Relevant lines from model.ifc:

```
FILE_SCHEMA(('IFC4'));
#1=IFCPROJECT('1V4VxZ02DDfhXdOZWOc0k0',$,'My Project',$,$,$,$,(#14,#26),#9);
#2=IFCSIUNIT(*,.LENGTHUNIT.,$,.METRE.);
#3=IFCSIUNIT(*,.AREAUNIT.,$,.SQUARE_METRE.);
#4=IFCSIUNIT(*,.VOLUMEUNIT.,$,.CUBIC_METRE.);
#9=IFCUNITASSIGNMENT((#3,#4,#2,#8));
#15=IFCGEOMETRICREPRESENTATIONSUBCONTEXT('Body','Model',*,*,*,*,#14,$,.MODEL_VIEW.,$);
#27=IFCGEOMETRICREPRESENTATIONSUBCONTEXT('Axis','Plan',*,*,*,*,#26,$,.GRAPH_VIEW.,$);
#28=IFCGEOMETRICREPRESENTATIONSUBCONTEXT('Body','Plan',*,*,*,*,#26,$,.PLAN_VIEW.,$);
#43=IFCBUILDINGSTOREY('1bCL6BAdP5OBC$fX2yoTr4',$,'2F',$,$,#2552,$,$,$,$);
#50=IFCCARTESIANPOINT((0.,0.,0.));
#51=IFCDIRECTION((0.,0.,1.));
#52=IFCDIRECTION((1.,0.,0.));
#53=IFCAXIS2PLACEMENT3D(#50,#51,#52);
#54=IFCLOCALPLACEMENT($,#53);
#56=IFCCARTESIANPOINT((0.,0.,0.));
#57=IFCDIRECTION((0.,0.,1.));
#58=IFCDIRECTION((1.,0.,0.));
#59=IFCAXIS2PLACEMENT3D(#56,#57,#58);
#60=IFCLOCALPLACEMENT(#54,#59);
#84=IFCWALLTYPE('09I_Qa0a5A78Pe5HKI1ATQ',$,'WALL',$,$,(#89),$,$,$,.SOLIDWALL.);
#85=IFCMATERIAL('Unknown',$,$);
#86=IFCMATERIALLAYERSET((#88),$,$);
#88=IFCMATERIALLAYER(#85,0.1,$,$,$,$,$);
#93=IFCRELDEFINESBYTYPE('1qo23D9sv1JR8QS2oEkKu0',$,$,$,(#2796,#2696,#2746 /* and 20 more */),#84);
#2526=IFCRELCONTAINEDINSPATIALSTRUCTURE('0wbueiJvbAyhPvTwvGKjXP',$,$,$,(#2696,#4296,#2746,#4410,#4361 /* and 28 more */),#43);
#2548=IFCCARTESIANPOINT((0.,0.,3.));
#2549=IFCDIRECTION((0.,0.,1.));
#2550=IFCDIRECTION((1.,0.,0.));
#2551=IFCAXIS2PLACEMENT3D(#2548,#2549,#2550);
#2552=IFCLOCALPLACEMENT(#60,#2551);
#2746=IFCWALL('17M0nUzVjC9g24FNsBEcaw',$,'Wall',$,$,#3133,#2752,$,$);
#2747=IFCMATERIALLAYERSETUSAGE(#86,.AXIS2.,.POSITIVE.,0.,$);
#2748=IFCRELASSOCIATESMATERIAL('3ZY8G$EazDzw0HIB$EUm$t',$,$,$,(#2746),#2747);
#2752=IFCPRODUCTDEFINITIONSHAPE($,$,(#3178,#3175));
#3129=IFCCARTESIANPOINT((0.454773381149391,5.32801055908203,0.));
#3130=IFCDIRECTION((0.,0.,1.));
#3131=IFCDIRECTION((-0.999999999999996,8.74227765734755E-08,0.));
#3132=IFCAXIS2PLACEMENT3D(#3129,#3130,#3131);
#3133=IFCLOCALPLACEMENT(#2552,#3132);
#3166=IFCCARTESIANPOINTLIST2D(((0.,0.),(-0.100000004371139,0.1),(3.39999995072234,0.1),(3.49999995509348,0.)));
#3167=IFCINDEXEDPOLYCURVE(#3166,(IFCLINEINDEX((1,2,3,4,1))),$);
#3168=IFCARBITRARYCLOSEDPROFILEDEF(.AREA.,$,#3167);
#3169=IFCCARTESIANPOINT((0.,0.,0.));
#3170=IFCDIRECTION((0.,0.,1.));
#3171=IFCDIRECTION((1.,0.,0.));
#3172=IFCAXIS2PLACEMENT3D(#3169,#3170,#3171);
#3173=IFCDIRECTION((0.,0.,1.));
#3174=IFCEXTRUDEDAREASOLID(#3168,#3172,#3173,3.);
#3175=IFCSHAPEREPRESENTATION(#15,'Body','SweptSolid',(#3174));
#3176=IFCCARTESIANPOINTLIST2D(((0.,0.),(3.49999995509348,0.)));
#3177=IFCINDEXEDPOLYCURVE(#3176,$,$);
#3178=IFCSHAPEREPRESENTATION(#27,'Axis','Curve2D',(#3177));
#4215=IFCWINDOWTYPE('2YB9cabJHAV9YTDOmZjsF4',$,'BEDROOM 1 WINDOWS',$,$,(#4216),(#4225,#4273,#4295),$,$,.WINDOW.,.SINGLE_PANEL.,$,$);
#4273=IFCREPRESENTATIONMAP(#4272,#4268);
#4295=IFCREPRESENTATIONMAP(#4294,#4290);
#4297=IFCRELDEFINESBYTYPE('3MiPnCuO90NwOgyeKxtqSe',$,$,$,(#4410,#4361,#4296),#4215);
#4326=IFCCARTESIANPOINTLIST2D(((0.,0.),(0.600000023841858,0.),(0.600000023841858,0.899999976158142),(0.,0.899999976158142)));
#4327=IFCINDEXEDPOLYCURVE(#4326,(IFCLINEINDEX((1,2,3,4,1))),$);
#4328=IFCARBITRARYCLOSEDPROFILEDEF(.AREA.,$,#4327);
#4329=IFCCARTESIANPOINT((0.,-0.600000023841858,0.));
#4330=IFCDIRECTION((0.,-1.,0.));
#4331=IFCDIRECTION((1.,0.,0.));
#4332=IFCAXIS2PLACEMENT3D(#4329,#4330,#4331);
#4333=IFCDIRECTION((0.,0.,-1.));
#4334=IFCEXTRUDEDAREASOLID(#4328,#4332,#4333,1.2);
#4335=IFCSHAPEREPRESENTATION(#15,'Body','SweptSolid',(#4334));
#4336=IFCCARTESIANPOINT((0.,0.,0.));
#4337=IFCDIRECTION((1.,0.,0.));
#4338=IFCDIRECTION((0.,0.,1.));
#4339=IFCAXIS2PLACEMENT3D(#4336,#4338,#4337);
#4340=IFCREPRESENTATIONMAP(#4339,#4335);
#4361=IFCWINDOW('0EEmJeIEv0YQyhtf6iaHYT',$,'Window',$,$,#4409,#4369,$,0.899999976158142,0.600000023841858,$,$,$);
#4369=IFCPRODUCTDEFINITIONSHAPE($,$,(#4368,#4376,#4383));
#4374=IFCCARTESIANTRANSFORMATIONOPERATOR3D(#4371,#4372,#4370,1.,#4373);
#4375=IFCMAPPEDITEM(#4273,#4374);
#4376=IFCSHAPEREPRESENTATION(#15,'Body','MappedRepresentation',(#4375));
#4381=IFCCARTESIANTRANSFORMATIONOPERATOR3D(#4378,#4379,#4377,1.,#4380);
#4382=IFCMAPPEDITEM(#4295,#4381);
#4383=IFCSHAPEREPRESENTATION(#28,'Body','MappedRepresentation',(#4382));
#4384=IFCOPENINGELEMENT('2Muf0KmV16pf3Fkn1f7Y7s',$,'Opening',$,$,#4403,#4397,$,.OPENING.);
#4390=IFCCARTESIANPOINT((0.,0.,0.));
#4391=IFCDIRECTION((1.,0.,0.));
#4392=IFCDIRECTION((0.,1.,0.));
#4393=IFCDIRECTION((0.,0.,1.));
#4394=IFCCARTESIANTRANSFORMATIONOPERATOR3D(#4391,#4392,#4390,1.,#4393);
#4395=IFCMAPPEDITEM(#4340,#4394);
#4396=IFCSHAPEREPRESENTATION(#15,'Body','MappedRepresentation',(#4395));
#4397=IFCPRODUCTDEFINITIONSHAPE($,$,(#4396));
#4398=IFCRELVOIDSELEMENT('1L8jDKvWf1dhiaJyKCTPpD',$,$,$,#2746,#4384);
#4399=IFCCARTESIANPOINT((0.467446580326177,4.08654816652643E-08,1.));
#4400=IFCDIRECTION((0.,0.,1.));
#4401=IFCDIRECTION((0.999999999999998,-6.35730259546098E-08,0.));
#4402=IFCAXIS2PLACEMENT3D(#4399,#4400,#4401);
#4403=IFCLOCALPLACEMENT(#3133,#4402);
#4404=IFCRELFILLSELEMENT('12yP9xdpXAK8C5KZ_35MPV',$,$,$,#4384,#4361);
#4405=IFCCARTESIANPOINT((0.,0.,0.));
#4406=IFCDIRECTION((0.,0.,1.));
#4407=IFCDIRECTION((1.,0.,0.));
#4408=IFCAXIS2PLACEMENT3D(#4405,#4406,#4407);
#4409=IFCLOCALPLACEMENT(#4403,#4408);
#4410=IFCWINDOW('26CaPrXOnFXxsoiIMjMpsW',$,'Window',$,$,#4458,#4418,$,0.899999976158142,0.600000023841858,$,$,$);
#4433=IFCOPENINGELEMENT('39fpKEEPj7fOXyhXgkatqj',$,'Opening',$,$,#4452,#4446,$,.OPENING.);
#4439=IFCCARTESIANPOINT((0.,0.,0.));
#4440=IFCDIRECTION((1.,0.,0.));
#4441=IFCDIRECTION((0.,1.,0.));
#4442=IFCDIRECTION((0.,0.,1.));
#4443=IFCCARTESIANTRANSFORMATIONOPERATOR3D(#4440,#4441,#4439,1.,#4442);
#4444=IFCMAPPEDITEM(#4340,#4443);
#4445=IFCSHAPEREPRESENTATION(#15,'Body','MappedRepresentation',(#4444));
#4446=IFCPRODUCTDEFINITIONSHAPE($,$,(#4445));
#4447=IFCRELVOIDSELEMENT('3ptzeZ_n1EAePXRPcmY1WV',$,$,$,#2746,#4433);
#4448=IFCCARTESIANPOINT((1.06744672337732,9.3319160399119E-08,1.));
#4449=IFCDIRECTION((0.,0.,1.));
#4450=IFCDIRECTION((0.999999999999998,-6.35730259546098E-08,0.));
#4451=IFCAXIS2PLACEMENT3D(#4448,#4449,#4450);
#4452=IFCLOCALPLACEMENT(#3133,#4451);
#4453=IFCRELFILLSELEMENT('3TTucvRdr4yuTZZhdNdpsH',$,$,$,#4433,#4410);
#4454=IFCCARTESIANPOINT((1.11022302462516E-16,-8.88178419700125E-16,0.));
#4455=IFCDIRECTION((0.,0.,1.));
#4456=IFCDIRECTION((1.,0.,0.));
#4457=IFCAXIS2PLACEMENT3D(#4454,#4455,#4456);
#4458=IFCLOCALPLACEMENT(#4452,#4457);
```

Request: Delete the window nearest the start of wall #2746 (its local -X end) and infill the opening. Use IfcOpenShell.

```python
import ifcopenshell
import ifcopenshell.api.feature
import ifcopenshell.api.root
import ifcopenshell.geom
import ifcopenshell.util.shape

model = ifcopenshell.open("model.ifc")
settings = ifcopenshell.geom.settings()


def volume(element):
    """Net volume in cubic metres, openings subtracted."""
    shape = ifcopenshell.geom.create_shape(settings, element)
    return ifcopenshell.util.shape.get_volume(shape.geometry)


window = model.by_guid("0EEmJeIEv0YQyhtf6iaHYT")
opening = window.FillsVoids[0].RelatingOpeningElement
wall = opening.VoidsElements[0].RelatingBuildingElement
before = volume(wall)

ifcopenshell.api.root.remove_product(model, product=window)
ifcopenshell.api.feature.remove_feature(model, feature=opening)

after = volume(wall)

print(f"wall volume {before:.3f} -> {after:.3f} m3")

model.write("model_v2.ifc")
```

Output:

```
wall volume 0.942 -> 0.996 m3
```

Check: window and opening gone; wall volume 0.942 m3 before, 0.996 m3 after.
